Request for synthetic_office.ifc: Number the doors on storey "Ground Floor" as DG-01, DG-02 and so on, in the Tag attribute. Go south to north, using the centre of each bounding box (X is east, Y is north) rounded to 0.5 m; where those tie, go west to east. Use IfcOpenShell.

First a look at what the model holds.

```python
import ifcopenshell
import ifcopenshell.util.element
import ifcopenshell.util.placement

model = ifcopenshell.open("synthetic_office.ifc")
print(model.schema)
storey = next(s for s in model.by_type("IfcBuildingStorey") if s.Name == "Ground Floor")
doors = [e for e in ifcopenshell.util.element.get_decomposition(storey) if e.is_a("IfcDoor")]
for e in sorted(doors, key=lambda e: e.id()):
    origin = ifcopenshell.util.placement.get_local_placement(e.ObjectPlacement)[:3, 3]
    print(e.id(), e.Tag, e.Name, origin.round(2) + 0.0, sep=" | ")
```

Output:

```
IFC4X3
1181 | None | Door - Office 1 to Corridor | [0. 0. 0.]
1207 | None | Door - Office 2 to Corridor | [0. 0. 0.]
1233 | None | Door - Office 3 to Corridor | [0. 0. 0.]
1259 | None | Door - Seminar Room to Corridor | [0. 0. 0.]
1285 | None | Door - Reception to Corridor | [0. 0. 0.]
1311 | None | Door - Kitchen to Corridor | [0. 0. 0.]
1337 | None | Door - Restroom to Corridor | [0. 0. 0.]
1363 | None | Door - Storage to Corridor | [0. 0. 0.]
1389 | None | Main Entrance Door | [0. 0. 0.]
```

```python
import ifcopenshell
import ifcopenshell.geom
import ifcopenshell.util.element
import ifcopenshell.util.shape

model = ifcopenshell.open("synthetic_office.ifc")
settings = ifcopenshell.geom.settings()
settings.set("use-world-coords", True)


def centre(element):
    shape = ifcopenshell.geom.create_shape(settings, element)
    return ifcopenshell.util.shape.get_bbox_centroid(shape.geometry)


storey = next(s for s in model.by_type("IfcBuildingStorey") if s.Name == "Ground Floor")
doors = [e for e in ifcopenshell.util.element.get_decomposition(storey) if e.is_a("IfcDoor")]

# Insertion points can sit at a corner or the storey origin, so sort by the geometry (in metres).
centres = {e: centre(e) for e in doors}
doors.sort(key=lambda e: (round(centres[e][1] / 0.5), centres[e][0]))

for i, e in enumerate(doors, start=1):
    number = f"DG-{i:02d}"
    e.Tag = number
    print(e.id(), number)

model.write("synthetic_office_rev.ifc")
```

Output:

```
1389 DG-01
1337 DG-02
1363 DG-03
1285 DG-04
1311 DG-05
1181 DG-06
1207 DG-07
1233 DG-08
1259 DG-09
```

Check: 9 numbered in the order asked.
